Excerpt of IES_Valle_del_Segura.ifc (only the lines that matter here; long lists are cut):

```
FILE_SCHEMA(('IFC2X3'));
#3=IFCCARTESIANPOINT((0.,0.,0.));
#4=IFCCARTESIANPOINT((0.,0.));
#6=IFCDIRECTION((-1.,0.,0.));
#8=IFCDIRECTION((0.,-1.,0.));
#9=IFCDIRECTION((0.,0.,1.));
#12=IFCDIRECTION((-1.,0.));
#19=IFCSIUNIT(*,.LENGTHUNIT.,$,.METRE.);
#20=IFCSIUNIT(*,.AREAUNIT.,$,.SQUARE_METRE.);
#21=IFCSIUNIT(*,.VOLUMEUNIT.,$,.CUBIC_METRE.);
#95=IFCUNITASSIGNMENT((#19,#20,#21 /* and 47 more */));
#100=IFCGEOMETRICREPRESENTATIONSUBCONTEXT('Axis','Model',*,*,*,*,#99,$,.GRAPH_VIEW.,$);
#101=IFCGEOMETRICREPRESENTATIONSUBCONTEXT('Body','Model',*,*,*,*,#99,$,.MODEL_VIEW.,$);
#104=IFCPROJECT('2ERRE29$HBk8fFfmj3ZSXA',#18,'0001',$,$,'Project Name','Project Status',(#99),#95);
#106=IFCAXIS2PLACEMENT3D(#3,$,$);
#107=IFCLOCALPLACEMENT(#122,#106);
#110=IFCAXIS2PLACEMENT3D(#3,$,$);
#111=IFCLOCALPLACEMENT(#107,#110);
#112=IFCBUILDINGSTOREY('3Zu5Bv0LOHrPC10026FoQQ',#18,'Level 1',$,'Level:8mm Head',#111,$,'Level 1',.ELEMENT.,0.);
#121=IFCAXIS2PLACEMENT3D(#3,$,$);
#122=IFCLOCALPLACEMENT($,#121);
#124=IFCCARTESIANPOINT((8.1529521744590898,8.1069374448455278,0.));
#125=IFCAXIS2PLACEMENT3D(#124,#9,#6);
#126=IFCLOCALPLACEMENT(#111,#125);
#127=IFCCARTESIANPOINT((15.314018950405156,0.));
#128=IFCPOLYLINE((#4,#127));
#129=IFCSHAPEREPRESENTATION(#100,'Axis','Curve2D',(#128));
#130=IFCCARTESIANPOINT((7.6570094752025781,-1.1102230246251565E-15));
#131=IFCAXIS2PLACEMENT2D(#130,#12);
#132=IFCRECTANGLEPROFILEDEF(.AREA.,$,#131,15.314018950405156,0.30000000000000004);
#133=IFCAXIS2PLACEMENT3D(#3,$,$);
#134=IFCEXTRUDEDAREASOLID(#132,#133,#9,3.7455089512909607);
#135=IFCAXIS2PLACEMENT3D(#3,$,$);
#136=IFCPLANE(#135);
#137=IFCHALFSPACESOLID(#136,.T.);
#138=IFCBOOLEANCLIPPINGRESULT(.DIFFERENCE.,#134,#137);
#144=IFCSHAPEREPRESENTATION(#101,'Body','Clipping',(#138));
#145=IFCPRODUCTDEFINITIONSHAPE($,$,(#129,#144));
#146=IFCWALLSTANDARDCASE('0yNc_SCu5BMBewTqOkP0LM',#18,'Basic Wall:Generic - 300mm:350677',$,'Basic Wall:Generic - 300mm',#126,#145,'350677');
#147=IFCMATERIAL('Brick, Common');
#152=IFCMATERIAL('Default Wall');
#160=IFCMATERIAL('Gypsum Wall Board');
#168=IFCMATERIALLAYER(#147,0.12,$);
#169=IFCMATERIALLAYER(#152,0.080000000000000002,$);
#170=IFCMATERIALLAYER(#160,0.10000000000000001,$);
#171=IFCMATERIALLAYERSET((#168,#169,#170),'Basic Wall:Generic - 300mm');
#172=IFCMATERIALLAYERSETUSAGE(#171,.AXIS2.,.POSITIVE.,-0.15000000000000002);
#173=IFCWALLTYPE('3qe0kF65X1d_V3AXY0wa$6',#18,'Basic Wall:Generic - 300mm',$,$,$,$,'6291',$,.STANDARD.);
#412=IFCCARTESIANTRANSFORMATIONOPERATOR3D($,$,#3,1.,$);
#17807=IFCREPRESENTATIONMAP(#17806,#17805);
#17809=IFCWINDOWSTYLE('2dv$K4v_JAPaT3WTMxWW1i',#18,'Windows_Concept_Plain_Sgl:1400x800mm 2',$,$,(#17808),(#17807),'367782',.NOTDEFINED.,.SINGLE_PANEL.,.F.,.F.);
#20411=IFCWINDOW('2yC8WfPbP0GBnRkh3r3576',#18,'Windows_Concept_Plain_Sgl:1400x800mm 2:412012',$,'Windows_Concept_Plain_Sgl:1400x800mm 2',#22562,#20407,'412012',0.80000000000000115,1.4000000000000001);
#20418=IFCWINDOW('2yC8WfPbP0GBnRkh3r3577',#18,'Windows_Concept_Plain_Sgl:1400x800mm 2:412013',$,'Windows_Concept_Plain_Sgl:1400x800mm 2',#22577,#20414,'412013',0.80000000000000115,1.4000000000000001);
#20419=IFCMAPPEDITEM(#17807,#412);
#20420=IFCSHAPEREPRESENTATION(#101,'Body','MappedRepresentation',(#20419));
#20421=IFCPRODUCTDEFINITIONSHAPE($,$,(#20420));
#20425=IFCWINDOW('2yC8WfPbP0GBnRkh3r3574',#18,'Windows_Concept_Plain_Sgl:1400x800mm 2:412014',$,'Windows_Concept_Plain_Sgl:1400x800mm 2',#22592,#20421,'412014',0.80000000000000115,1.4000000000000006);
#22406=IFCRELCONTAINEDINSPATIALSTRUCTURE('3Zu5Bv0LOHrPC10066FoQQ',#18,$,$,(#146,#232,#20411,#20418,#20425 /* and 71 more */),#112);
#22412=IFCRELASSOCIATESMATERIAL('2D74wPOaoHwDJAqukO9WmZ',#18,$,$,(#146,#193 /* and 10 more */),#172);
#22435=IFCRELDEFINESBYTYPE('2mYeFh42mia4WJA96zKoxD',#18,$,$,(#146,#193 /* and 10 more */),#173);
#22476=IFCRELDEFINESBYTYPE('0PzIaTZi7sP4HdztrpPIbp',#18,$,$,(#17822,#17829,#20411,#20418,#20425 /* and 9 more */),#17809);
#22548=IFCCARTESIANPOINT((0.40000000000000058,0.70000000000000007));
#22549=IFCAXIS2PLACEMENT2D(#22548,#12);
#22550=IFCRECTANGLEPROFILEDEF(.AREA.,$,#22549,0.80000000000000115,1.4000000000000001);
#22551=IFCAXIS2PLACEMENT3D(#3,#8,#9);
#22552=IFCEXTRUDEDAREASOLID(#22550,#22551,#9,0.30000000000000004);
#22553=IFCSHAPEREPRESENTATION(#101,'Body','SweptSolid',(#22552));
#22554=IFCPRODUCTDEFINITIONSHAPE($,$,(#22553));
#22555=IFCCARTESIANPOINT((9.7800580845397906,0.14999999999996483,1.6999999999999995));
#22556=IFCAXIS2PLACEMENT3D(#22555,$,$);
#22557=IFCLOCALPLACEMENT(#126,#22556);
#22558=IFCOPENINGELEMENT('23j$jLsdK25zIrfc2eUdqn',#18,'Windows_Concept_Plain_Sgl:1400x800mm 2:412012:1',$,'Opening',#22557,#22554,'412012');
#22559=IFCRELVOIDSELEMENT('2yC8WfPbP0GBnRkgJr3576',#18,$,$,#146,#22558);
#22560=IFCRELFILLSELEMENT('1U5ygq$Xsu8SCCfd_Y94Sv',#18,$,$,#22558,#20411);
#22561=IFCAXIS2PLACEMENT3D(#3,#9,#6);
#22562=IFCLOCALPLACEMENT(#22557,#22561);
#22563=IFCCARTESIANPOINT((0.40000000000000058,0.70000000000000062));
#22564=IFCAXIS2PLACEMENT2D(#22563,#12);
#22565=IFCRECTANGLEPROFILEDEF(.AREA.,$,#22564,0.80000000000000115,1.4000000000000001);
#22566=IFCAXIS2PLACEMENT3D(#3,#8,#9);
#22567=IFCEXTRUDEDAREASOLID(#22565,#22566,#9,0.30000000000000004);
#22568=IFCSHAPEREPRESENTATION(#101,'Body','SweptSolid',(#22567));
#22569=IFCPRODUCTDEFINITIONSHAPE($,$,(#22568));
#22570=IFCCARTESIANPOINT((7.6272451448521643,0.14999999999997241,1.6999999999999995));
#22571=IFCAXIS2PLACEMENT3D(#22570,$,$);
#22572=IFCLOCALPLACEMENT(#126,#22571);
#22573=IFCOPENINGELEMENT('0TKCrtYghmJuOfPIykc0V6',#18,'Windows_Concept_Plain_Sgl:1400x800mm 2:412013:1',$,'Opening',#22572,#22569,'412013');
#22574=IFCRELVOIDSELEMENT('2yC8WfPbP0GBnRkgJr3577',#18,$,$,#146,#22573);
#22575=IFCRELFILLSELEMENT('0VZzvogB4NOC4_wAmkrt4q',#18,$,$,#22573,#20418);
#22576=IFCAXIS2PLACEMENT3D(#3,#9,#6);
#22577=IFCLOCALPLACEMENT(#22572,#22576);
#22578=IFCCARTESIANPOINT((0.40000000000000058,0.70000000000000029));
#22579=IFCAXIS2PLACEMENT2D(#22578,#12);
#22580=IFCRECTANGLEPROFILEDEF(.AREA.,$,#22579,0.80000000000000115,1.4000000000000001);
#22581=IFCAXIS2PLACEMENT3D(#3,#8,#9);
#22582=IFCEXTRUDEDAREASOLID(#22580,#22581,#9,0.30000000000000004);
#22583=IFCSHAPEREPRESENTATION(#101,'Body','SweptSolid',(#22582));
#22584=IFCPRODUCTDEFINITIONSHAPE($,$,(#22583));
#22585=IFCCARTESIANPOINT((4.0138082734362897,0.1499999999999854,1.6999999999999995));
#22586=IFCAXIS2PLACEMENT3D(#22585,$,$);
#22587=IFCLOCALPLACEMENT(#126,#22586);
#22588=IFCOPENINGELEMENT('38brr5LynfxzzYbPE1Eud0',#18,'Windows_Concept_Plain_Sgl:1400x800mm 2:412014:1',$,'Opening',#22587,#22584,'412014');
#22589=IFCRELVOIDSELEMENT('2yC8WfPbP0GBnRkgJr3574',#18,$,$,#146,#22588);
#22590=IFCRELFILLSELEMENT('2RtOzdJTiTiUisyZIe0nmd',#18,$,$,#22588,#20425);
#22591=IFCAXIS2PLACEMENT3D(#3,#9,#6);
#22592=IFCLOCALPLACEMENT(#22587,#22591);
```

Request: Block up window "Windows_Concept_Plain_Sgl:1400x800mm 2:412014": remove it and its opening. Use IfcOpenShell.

```python
import ifcopenshell
import ifcopenshell.api.feature
import ifcopenshell.api.root
import ifcopenshell.geom
import ifcopenshell.util.shape

model = ifcopenshell.open("IES_Valle_del_Segura.ifc")
settings = ifcopenshell.geom.settings()


def volume(element):
    """Net volume in cubic metres, openings subtracted."""
    shape = ifcopenshell.geom.create_shape(settings, element)
    return ifcopenshell.util.shape.get_volume(shape.geometry)


window = model.by_guid("2yC8WfPbP0GBnRkh3r3574")
opening = window.FillsVoids[0].RelatingOpeningElement
wall = opening.VoidsElements[0].RelatingBuildingElement
before = volume(wall)

ifcopenshell.api.root.remove_product(model, product=window)
ifcopenshell.api.feature.remove_feature(model, feature=opening)

after = volume(wall)

print(f"wall volume {before:.3f} -> {after:.3f} m3")

model.write("IES_Valle_del_Segura-out.ifc")
```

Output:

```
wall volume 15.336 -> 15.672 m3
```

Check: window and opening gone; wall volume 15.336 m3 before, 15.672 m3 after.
